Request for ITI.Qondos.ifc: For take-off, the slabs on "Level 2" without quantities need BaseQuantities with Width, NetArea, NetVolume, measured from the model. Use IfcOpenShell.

First a look at what the model holds.

```python
import ifcopenshell
import ifcopenshell.util.element
import ifcopenshell.util.unit

model = ifcopenshell.open("ITI.Qondos.ifc")
print(model.schema)
for unit_type in ("LENGTHUNIT", "AREAUNIT", "VOLUMEUNIT"):
    print(unit_type, ifcopenshell.util.unit.calculate_unit_scale(model, unit_type))
storey = next(s for s in model.by_type("IfcBuildingStorey") if s.Name == "Level 2")
slabs = [e for e in ifcopenshell.util.element.get_decomposition(storey) if e.is_a("IfcSlab")]
for e in sorted(slabs, key=lambda e: e.id()):
    print(e.id(), e.is_a(), e.Name, list(ifcopenshell.util.element.get_psets(e, qtos_only=True)), sep=" | ")
```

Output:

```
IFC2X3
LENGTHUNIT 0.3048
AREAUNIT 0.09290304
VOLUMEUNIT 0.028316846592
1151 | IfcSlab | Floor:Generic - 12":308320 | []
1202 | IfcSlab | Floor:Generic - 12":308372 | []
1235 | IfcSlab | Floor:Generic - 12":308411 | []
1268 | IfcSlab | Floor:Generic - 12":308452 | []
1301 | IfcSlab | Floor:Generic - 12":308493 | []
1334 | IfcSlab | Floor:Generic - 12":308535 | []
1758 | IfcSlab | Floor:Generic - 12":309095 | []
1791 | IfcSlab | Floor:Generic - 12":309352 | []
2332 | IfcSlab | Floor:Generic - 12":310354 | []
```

```python
import ifcopenshell
import ifcopenshell.api.pset
import ifcopenshell.geom
import ifcopenshell.util.element
import ifcopenshell.util.shape
import ifcopenshell.util.unit

model = ifcopenshell.open("ITI.Qondos.ifc")
unit_scale = ifcopenshell.util.unit.calculate_unit_scale(model)
area_scale = ifcopenshell.util.unit.calculate_unit_scale(model, "AREAUNIT")
volume_scale = ifcopenshell.util.unit.calculate_unit_scale(model, "VOLUMEUNIT")
settings = ifcopenshell.geom.settings()

storey = next(s for s in model.by_type("IfcBuildingStorey") if s.Name == "Level 2")
slabs = [e for e in ifcopenshell.util.element.get_decomposition(storey) if e.is_a("IfcSlab")]

for e in sorted(slabs, key=lambda e: e.id()):
    if ifcopenshell.util.element.get_psets(e, qtos_only=True, should_inherit=False):
        continue
    # Geometry comes back in metres, in the element's own axes.
    shape = ifcopenshell.geom.create_shape(settings, e)
    values = {
        "Width": ifcopenshell.util.shape.get_z(shape.geometry) / unit_scale,
        "NetArea": ifcopenshell.util.shape.get_footprint_area(shape.geometry) / area_scale,
        "NetVolume": ifcopenshell.util.shape.get_volume(shape.geometry) / volume_scale,
    }
    qto = ifcopenshell.api.pset.add_qto(model, product=e, name="BaseQuantities")
    ifcopenshell.api.pset.edit_qto(model, qto=qto, properties=values)
    print(e.id(), {k: round(v, 3) for k, v in values.items()})

model.write("ITI.Qondos_v2.ifc")
```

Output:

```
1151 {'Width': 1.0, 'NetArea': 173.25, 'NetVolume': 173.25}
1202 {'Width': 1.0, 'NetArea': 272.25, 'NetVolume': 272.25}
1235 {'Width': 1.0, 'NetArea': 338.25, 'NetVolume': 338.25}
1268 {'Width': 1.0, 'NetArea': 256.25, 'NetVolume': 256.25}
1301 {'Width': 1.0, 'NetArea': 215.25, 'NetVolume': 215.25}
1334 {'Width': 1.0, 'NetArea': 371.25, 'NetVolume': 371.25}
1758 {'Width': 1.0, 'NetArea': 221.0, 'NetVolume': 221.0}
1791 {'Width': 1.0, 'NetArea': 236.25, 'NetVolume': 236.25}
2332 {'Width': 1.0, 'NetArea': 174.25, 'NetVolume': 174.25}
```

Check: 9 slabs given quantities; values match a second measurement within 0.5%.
